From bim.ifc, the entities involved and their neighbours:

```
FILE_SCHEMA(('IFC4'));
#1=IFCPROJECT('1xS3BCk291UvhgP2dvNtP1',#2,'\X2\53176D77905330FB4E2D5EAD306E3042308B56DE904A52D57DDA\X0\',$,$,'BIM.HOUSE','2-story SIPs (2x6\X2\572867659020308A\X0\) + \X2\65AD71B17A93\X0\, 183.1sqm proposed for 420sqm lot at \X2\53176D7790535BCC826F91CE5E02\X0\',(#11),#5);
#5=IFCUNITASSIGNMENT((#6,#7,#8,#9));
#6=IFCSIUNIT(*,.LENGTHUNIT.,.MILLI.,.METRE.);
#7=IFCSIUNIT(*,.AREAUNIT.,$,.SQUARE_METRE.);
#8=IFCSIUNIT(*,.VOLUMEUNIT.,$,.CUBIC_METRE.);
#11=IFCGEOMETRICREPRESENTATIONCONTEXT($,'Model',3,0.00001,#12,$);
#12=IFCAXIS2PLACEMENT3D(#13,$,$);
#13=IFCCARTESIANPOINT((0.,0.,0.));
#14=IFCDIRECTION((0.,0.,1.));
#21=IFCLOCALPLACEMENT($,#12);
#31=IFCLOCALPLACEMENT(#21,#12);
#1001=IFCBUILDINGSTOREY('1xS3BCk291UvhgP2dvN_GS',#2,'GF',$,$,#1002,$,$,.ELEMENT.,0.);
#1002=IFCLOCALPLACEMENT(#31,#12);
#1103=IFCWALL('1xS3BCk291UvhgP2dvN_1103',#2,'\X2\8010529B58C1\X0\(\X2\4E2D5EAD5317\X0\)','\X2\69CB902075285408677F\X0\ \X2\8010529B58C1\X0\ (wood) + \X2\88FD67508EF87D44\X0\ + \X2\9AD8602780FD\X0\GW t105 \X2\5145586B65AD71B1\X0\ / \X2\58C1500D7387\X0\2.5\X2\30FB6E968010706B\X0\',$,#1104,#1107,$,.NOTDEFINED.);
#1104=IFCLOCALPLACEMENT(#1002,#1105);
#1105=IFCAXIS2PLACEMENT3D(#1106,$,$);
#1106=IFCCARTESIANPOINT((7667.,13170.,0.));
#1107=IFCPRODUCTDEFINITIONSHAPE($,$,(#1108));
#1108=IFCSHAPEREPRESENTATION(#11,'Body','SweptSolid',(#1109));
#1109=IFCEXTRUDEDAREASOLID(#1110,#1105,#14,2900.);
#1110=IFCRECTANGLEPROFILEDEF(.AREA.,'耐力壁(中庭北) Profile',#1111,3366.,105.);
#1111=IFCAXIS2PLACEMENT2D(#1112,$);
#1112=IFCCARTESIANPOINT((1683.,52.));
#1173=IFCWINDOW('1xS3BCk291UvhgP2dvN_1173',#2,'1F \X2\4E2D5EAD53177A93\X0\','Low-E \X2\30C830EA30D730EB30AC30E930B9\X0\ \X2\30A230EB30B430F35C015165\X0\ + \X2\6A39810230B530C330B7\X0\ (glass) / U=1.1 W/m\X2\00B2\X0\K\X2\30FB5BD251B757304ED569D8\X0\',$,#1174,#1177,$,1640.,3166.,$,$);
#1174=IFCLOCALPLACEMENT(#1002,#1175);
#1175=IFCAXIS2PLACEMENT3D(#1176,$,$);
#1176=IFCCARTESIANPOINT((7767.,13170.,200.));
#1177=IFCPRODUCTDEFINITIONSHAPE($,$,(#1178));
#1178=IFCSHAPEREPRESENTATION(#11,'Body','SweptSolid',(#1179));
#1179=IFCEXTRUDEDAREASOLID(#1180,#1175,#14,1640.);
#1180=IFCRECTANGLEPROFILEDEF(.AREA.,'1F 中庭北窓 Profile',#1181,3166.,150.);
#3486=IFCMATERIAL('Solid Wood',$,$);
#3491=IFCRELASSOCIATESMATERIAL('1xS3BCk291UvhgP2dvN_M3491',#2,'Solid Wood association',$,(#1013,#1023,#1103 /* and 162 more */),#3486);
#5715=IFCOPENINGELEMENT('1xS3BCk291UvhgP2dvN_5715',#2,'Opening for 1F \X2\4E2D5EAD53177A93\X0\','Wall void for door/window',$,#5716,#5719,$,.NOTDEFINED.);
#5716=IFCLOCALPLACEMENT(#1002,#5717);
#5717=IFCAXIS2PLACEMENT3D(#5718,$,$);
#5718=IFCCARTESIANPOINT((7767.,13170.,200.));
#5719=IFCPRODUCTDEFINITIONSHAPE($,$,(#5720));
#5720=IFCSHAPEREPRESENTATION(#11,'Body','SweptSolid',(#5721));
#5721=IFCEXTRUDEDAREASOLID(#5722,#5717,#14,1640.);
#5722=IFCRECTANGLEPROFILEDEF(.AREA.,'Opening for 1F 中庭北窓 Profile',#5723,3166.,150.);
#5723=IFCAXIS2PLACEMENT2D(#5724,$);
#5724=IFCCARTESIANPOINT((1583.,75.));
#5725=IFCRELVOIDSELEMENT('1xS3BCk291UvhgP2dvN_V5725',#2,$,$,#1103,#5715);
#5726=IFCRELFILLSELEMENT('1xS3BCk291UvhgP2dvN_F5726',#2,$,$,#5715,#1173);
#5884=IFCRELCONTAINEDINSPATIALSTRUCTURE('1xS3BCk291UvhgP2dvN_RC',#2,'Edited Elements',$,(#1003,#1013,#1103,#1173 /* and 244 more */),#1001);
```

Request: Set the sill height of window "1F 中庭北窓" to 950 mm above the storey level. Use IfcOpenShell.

```python
import numpy as np
import ifcopenshell
import ifcopenshell.api.geometry
import ifcopenshell.geom
import ifcopenshell.util.element
import ifcopenshell.util.placement
import ifcopenshell.util.shape
import ifcopenshell.util.unit

model = ifcopenshell.open("bim.ifc")
unit_scale = ifcopenshell.util.unit.calculate_unit_scale(model)

window = model.by_guid("1xS3BCk291UvhgP2dvN_1173")
opening = window.FillsVoids[0].RelatingOpeningElement
storey = ifcopenshell.util.element.get_container(window, ifc_class="IfcBuildingStorey")
level = ifcopenshell.util.placement.get_local_placement(storey.ObjectPlacement)[2, 3]

# The opening's origin need not be at the sill, so measure its lowest point.
shape = ifcopenshell.geom.create_shape(ifcopenshell.geom.settings(), opening)
bottom = ifcopenshell.util.shape.get_shape_bottom_elevation(shape, shape.geometry) / unit_scale
dz = level + 950.0 - bottom

shift = np.array([0.0, 0.0, dz])
# The window is not placed relative to its opening, so move both.
for product in (opening, window):
    matrix = ifcopenshell.util.placement.get_local_placement(product.ObjectPlacement)
    matrix[:3, 3] += shift
    ifcopenshell.api.geometry.edit_object_placement(model, product=product, matrix=matrix, is_si=False)

print(f"moved by {dz * unit_scale:+.3f} m")

model.write("bim_updated.ifc")
```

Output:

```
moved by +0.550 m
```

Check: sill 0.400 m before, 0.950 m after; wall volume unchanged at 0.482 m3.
